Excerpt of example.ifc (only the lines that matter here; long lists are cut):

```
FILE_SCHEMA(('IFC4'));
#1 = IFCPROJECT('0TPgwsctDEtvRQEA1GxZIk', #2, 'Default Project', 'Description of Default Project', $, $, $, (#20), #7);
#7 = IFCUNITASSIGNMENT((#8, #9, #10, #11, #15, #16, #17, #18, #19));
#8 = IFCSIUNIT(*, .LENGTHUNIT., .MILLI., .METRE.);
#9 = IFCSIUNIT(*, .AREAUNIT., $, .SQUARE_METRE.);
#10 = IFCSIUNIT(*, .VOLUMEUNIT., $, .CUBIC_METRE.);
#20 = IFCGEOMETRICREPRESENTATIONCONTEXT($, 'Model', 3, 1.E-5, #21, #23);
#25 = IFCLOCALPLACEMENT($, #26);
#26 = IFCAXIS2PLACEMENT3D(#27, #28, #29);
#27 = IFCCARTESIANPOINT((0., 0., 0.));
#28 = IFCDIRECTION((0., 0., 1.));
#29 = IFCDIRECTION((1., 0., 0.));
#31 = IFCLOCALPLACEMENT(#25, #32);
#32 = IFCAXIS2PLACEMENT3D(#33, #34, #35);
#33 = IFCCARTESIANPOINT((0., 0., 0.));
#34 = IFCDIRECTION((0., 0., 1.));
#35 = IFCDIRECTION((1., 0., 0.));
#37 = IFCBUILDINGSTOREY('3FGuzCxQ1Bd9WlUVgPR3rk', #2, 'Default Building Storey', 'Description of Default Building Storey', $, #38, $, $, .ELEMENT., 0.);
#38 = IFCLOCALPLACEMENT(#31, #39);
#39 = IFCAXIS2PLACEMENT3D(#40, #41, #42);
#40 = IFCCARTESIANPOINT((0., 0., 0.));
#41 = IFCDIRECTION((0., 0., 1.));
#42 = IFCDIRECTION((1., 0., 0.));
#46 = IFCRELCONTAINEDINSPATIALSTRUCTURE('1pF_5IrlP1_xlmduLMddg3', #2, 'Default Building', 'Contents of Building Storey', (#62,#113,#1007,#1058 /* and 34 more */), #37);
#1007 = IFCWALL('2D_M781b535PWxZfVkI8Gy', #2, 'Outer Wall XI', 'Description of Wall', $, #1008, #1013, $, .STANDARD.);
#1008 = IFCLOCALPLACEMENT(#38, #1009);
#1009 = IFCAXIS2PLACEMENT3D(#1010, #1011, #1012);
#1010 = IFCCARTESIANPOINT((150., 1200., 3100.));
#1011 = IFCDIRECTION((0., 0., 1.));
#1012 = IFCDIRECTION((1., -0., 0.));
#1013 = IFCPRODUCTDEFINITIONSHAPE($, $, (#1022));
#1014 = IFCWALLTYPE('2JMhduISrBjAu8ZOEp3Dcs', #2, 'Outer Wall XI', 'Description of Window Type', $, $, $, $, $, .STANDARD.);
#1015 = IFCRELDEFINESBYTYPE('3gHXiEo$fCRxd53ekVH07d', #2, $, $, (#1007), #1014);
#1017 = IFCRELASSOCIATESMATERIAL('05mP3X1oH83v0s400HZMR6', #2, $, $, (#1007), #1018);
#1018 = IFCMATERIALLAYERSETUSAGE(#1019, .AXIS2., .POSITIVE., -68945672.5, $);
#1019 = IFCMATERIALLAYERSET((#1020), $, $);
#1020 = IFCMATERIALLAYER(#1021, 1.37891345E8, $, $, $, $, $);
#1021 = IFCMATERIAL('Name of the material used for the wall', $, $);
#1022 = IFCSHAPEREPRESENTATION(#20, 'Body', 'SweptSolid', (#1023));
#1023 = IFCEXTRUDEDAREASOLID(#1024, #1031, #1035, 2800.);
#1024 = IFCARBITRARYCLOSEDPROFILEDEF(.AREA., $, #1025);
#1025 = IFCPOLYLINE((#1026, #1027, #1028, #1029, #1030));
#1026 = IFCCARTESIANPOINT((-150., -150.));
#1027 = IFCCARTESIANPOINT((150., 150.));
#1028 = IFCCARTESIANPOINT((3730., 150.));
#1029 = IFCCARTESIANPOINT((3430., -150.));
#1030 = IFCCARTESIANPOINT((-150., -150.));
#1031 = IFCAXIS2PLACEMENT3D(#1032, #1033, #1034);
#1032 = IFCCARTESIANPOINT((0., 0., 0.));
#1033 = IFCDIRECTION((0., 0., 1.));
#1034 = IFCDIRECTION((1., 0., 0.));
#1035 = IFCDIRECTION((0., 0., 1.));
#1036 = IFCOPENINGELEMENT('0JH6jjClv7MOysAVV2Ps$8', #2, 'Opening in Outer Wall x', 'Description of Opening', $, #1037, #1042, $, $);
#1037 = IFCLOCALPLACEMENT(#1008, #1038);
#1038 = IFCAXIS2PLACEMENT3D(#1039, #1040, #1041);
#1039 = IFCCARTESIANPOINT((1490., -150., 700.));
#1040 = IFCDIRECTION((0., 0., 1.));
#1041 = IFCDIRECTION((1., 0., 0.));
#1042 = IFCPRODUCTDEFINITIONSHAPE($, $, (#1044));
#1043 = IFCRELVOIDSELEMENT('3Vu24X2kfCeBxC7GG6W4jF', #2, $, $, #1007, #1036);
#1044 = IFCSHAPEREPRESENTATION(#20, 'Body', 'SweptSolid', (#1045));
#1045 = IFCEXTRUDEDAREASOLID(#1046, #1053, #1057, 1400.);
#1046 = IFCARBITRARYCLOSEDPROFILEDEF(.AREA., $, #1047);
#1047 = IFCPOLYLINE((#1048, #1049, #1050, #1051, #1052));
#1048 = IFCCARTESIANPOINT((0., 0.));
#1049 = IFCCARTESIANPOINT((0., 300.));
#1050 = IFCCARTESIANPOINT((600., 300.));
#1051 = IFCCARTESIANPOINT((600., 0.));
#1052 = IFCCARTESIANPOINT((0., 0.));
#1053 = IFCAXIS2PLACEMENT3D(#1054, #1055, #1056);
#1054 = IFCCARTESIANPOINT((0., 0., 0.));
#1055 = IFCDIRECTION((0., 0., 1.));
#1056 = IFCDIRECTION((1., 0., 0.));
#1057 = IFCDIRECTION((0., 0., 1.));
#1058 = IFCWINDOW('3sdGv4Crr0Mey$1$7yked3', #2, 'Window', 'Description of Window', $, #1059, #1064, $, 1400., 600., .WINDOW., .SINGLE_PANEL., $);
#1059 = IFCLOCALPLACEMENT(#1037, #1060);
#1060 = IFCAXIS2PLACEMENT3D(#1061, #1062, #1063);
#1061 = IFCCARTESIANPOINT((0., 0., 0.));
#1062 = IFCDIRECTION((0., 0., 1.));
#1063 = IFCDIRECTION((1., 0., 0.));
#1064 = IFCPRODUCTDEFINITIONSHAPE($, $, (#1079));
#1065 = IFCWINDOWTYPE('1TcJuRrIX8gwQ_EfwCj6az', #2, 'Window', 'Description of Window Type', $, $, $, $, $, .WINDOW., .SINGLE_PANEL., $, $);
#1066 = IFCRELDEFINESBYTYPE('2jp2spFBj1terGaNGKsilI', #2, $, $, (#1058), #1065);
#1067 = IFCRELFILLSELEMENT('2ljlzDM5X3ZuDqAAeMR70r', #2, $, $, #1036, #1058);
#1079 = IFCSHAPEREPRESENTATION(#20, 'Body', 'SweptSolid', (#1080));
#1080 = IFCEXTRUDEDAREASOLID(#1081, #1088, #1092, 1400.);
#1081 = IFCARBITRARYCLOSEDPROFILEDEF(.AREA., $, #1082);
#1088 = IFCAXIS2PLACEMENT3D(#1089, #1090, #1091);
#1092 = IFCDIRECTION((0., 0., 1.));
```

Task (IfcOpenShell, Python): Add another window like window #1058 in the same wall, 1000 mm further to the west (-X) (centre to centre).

```python
import ifcopenshell
import ifcopenshell.api.feature
import ifcopenshell.api.geometry
import ifcopenshell.api.root
import ifcopenshell.geom
import ifcopenshell.util.element
import ifcopenshell.util.placement
import ifcopenshell.util.shape
import ifcopenshell.util.unit

model = ifcopenshell.open("example.ifc")
unit_scale = ifcopenshell.util.unit.calculate_unit_scale(model)
settings = ifcopenshell.geom.settings()


def volume(element):
    """Net volume in cubic metres, openings subtracted."""
    shape = ifcopenshell.geom.create_shape(settings, element)
    return ifcopenshell.util.shape.get_volume(shape.geometry)


def reuse_history(source, copy):
    """copy_class also copies each property set's owner history, people and application; keep the originals."""
    for rel in copy.IsDefinedBy:
        if rel.is_a("IfcRelDefinesByProperties") and (history := rel.RelatingPropertyDefinition.OwnerHistory):
            rel.RelatingPropertyDefinition.OwnerHistory = source.OwnerHistory
            ifcopenshell.util.element.remove_deep2(model, history)


window = model.by_guid("3sdGv4Crr0Mey$1$7yked3")
opening = window.FillsVoids[0].RelatingOpeningElement
wall = opening.VoidsElements[0].RelatingBuildingElement
before = volume(wall)
shift = ifcopenshell.util.placement.get_local_placement(wall.ObjectPlacement)[:3, 0] * -1 / unit_scale

# copy_class copies the void relationship, type, container and properties, but no geometry.
new_opening = ifcopenshell.api.root.copy_class(model, product=opening)
new_opening.Representation = ifcopenshell.util.element.copy_deep(
    model, opening.Representation, exclude=["IfcGeometricRepresentationContext", "IfcRepresentationMap"]
)
new_window = ifcopenshell.api.root.copy_class(model, product=window)
new_window.Representation = ifcopenshell.util.element.copy_deep(
    model, window.Representation, exclude=["IfcGeometricRepresentationContext", "IfcRepresentationMap"]
)
reuse_history(window, new_window)
ifcopenshell.api.feature.add_filling(model, opening=new_opening, element=new_window)

for old, new in ((opening, new_opening), (window, new_window)):
    matrix = ifcopenshell.util.placement.get_local_placement(old.ObjectPlacement)
    matrix[:3, 3] += shift
    ifcopenshell.api.geometry.edit_object_placement(model, product=new, matrix=matrix, is_si=False)

after = volume(wall)

print(f"wall volume {before:.3f} -> {after:.3f} m3")

model.write("example_rev.ifc")
```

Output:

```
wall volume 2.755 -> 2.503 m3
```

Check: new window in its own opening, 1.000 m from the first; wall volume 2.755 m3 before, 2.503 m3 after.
